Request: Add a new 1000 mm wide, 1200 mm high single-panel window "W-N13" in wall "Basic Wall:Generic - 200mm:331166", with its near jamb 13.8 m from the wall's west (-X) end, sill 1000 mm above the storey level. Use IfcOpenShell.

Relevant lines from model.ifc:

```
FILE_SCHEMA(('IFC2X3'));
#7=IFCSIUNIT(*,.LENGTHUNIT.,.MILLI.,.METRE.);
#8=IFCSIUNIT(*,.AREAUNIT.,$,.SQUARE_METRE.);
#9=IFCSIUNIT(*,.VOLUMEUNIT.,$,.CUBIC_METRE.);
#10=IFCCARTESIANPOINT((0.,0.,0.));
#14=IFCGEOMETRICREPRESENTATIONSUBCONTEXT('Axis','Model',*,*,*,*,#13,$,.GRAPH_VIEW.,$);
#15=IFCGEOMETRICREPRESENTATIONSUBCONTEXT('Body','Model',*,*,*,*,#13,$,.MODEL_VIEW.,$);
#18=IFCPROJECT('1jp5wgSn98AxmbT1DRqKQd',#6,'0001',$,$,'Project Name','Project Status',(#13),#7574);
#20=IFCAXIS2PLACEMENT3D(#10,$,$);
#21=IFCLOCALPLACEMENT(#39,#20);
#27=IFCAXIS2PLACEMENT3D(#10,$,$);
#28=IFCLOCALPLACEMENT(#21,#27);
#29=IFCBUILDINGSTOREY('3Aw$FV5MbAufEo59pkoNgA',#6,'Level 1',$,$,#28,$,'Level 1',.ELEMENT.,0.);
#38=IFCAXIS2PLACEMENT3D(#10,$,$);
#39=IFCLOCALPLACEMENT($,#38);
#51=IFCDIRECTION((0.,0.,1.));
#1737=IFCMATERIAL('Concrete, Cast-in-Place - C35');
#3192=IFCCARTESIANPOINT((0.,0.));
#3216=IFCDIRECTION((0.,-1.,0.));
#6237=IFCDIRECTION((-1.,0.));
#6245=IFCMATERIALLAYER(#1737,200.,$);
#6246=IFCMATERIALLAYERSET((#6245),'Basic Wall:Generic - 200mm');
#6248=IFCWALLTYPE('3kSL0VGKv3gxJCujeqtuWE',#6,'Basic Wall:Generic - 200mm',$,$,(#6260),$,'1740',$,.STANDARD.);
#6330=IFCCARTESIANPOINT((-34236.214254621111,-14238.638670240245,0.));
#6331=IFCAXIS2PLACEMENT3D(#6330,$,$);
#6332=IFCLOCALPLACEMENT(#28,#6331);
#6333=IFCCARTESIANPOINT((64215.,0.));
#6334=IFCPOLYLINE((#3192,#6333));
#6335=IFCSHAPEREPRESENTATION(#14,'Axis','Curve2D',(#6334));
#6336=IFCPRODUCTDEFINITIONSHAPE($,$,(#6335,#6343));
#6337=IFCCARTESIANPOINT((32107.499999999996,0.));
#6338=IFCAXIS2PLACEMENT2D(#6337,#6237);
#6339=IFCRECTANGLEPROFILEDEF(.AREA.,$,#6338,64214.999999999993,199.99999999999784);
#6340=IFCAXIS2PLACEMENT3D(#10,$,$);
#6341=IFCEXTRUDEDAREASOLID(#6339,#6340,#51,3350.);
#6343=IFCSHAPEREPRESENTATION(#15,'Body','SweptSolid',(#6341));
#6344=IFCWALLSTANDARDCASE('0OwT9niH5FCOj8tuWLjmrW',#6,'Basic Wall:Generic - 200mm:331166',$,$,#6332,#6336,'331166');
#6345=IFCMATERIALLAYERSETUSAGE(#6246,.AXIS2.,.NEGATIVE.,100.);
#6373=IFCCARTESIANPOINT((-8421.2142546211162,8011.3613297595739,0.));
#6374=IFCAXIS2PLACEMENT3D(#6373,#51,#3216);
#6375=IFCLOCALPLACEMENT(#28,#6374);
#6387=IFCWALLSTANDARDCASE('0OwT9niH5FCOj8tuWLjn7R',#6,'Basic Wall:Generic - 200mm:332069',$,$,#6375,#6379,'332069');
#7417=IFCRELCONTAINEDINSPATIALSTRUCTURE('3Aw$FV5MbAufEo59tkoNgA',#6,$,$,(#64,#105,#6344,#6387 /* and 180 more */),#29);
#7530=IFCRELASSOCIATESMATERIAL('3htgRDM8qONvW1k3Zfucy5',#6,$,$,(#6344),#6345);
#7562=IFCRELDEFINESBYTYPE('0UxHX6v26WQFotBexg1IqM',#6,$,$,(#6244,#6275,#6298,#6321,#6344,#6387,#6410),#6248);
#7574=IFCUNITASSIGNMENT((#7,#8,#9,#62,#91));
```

```python
import numpy as np
import ifcopenshell
import ifcopenshell.api.feature
import ifcopenshell.api.geometry
import ifcopenshell.api.root
import ifcopenshell.api.spatial
import ifcopenshell.api.type
import ifcopenshell.geom
import ifcopenshell.util.element
import ifcopenshell.util.placement
import ifcopenshell.util.representation
import ifcopenshell.util.shape
import ifcopenshell.util.unit

model = ifcopenshell.open("model.ifc")
unit_scale = ifcopenshell.util.unit.calculate_unit_scale(model)
settings = ifcopenshell.geom.settings()


def volume(element):
    """Net volume in cubic metres, openings subtracted."""
    shape = ifcopenshell.geom.create_shape(settings, element)
    return ifcopenshell.util.shape.get_volume(shape.geometry)


wall = model.by_id(6344)
storey = ifcopenshell.util.element.get_container(wall, ifc_class="IfcBuildingStorey")
context = ifcopenshell.util.representation.get_context(model, "Model", "Body", "MODEL_VIEW")
before = volume(wall)

width, height, from_end, sill = 1, 1.2, 13.8, 1  # metres

# The wall runs along its own X axis, and the end named is its -X end.
wall_shape = ifcopenshell.geom.create_shape(settings, wall)
x, y, z = ifcopenshell.util.shape.get_vertices(wall_shape.geometry).T
start = x.min() + from_end
face, thickness = float(y.min()), float(y.max() - y.min())
wall_matrix = ifcopenshell.util.placement.get_local_placement(wall.ObjectPlacement)
level = ifcopenshell.util.placement.get_local_placement(storey.ObjectPlacement)[2, 3]


def in_wall(x, y):
    """Placement at x, y metres in the wall's axes, at sill height."""
    matrix = wall_matrix.copy()
    matrix[:, 3] = wall_matrix @ np.array([x / unit_scale, y / unit_scale, 0.0, 1.0])
    matrix[2, 3] = level + sill / unit_scale
    return matrix


# Opening: a box that overshoots both wall faces by 50 mm.
opening = ifcopenshell.api.root.create_entity(model, ifc_class="IfcOpeningElement")
box = ifcopenshell.api.geometry.add_wall_representation(
    model, context=context, length=width, height=height, thickness=thickness + 0.1
)
ifcopenshell.api.geometry.assign_representation(model, product=opening, representation=box)
ifcopenshell.api.geometry.edit_object_placement(model, product=opening, matrix=in_wall(start, face - 0.05), is_si=False)
ifcopenshell.api.feature.add_feature(model, feature=opening, element=wall)

window = ifcopenshell.api.root.create_entity(model, ifc_class="IfcWindow", name="W-N13")
window.OverallWidth, window.OverallHeight = width / unit_scale, height / unit_scale
body = ifcopenshell.api.geometry.add_window_representation(
    model,
    context=context,
    overall_width=window.OverallWidth,
    overall_height=window.OverallHeight,
    partition_type="SINGLE_PANEL",
)
ifcopenshell.api.geometry.assign_representation(model, product=window, representation=body)
ifcopenshell.api.spatial.assign_container(model, products=[window], relating_structure=storey)
fills = ifcopenshell.api.feature.add_filling(model, opening=opening, element=window)
fills.OwnerHistory = window.OwnerHistory  # required in IFC2X3

# IFC2X3 keeps the operation on the window style.
style = ifcopenshell.api.root.create_entity(model, ifc_class="IfcWindowStyle", name="W-N13")
style.OperationType, style.ConstructionType = "SINGLE_PANEL", "NOTDEFINED"
style.ParameterTakesPrecedence = style.Sizeable = False
ifcopenshell.api.type.assign_type(model, related_objects=[window], relating_type=style)

# Centre the window in the wall's thickness.
ifcopenshell.api.geometry.edit_object_placement(model, product=window, matrix=in_wall(start, face), is_si=False)
window_shape = ifcopenshell.geom.create_shape(settings, window)
depth = ifcopenshell.util.shape.get_vertices(window_shape.geometry)[:, 1]
offset = face + thickness / 2 - (depth.min() + depth.max()) / 2
ifcopenshell.api.geometry.edit_object_placement(model, product=window, matrix=in_wall(start, offset), is_si=False)

after = volume(wall)

print(f"wall volume {before:.3f} -> {after:.3f} m3")

model.write("model_rev.ifc")
```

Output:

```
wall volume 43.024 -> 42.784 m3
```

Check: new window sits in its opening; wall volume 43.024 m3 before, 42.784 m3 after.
